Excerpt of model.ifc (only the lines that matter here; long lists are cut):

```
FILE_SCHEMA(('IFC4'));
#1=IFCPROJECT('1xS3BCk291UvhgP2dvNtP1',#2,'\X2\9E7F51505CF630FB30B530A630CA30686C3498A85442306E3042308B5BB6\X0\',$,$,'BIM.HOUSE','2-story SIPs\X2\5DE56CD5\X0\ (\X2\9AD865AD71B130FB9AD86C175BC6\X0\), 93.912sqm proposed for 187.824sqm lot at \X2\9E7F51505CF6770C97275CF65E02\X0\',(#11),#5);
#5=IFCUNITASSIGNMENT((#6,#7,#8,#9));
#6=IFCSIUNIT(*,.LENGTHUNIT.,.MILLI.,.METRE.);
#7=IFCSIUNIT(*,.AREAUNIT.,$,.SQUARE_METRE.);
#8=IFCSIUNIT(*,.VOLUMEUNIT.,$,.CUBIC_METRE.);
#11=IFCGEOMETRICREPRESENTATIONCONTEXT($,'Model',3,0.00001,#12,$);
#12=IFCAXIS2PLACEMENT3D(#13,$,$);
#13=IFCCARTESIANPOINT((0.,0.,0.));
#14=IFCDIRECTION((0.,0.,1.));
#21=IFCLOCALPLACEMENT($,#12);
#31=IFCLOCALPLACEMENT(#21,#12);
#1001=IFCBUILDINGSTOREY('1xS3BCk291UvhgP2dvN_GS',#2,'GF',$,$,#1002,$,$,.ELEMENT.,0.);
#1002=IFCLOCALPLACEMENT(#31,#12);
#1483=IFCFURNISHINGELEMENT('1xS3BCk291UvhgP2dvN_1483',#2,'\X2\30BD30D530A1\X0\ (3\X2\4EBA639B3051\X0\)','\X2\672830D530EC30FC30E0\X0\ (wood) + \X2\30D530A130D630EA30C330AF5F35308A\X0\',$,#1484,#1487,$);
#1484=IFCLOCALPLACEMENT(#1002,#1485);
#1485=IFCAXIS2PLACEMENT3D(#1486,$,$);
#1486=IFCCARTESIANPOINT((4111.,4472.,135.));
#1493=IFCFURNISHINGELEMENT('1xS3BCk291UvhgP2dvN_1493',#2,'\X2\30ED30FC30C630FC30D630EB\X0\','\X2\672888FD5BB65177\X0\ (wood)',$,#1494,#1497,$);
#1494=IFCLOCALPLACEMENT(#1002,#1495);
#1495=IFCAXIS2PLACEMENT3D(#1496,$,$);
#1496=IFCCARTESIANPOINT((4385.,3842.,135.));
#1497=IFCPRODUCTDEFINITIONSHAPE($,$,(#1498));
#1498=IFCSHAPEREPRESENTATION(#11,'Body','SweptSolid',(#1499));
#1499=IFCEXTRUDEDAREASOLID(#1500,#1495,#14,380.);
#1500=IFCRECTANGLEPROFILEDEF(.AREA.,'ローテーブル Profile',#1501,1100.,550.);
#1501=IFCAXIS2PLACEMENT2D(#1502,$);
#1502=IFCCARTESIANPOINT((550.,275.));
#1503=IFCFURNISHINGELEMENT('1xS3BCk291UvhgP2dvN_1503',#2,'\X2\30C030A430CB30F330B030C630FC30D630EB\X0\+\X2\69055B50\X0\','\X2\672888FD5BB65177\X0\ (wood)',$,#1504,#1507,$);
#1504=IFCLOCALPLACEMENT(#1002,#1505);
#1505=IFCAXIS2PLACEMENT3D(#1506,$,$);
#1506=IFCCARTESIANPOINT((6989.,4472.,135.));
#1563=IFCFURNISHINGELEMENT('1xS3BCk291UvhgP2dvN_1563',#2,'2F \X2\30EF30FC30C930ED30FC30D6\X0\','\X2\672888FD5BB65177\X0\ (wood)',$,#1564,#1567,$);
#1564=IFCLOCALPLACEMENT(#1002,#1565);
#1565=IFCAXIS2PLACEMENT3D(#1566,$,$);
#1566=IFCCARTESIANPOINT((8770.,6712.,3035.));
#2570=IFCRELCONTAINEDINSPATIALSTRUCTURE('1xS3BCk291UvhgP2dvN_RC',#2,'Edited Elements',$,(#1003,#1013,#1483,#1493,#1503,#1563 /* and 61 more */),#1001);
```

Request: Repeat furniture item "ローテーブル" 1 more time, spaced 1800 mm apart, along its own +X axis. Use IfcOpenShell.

```python
import ifcopenshell
import ifcopenshell.api.geometry
import ifcopenshell.api.root
import ifcopenshell.util.element
import ifcopenshell.util.placement

model = ifcopenshell.open("model.ifc")


def reuse_history(source, copy):
    """copy_class also copies each property set's owner history, people and application; keep the originals."""
    for rel in copy.IsDefinedBy:
        if rel.is_a("IfcRelDefinesByProperties") and (history := rel.RelatingPropertyDefinition.OwnerHistory):
            rel.RelatingPropertyDefinition.OwnerHistory = source.OwnerHistory
            ifcopenshell.util.element.remove_deep2(model, history)


source = model.by_id(1493)
base = ifcopenshell.util.placement.get_local_placement(source.ObjectPlacement)
step = base[:3, 0] * 1800.0

for i in range(1, 2):
    copy = ifcopenshell.api.root.copy_class(model, product=source)
    copy.Representation = ifcopenshell.util.element.copy_deep(
        model, source.Representation, exclude=["IfcGeometricRepresentationContext", "IfcRepresentationMap"]
    )
    reuse_history(source, copy)
    matrix = base.copy()
    matrix[:3, 3] += i * step
    print("added at", matrix[:3, 3].round(3) + 0.0)
    ifcopenshell.api.geometry.edit_object_placement(model, product=copy, matrix=matrix, is_si=False)

model.write("model_updated.ifc")
```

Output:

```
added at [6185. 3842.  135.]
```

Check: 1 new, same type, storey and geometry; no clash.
